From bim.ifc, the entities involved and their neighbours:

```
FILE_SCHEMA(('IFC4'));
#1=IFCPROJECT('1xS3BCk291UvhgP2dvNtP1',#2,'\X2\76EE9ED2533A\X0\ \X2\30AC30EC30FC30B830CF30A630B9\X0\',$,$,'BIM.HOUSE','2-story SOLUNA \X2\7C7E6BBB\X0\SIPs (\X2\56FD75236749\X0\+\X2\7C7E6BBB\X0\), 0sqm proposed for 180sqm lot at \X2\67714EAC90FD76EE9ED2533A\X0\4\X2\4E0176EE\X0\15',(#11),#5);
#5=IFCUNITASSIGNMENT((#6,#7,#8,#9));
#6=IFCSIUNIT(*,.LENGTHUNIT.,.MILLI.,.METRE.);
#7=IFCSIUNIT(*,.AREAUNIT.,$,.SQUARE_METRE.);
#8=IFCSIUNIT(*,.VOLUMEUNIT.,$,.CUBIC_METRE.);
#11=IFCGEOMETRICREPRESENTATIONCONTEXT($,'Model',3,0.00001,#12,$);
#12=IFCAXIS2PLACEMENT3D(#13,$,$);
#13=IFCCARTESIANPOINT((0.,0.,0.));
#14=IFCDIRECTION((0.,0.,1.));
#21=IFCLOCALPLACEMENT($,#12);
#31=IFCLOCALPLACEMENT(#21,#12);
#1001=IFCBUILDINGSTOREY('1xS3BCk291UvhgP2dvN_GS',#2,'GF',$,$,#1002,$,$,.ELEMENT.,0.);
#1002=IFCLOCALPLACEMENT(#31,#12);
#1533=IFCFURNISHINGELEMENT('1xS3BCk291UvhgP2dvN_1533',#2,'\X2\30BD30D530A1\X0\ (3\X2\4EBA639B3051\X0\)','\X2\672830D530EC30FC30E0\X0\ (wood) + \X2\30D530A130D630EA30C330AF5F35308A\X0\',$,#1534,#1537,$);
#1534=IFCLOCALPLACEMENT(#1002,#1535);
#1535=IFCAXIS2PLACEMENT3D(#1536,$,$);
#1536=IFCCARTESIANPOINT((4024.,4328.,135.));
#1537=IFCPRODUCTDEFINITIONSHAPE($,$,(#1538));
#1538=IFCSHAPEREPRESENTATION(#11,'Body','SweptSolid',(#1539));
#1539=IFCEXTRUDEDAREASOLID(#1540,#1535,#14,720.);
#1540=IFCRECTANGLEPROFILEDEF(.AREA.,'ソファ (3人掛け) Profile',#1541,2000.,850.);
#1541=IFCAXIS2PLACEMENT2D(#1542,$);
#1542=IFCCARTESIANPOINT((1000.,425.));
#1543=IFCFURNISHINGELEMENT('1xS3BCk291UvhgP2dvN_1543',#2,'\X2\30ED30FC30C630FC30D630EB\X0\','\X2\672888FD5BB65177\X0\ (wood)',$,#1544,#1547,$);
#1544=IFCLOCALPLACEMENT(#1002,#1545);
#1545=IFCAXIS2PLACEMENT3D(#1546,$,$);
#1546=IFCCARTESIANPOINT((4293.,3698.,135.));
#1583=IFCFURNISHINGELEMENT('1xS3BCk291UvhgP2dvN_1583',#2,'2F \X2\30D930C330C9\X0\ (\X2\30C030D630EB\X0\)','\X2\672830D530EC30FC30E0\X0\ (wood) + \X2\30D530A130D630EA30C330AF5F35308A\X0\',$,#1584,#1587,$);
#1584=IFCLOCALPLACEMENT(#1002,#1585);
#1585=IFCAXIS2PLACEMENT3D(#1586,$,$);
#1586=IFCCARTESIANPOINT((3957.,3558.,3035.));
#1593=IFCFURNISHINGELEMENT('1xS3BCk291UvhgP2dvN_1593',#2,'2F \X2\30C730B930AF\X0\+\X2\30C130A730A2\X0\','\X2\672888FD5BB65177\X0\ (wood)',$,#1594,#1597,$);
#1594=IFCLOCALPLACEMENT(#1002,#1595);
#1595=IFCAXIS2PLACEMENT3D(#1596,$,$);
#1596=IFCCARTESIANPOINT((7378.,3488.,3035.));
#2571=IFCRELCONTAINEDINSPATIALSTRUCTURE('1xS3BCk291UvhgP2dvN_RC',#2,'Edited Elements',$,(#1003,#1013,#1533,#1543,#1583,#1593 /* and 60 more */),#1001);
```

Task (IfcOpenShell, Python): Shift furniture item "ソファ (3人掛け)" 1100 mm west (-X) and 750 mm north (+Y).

```python
import ifcopenshell
import ifcopenshell.api.geometry
import ifcopenshell.util.placement
import ifcopenshell.util.unit

model = ifcopenshell.open("bim.ifc")
unit_scale = ifcopenshell.util.unit.calculate_unit_scale(model)

item = model.by_guid("1xS3BCk291UvhgP2dvN_1533")
matrix = ifcopenshell.util.placement.get_local_placement(item.ObjectPlacement)
matrix[0, 3] -= 1.1 / unit_scale
matrix[1, 3] += 0.75 / unit_scale
ifcopenshell.api.geometry.edit_object_placement(model, product=item, matrix=matrix, is_si=False)

print(ifcopenshell.util.placement.get_local_placement(item.ObjectPlacement).round(3) + 0.0)

model.write("bim-out.ifc")
```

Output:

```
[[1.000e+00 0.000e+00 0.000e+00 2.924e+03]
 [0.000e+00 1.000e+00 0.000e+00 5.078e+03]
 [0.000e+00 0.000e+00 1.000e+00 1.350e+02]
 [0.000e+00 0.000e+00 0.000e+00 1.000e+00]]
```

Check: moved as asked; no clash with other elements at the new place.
